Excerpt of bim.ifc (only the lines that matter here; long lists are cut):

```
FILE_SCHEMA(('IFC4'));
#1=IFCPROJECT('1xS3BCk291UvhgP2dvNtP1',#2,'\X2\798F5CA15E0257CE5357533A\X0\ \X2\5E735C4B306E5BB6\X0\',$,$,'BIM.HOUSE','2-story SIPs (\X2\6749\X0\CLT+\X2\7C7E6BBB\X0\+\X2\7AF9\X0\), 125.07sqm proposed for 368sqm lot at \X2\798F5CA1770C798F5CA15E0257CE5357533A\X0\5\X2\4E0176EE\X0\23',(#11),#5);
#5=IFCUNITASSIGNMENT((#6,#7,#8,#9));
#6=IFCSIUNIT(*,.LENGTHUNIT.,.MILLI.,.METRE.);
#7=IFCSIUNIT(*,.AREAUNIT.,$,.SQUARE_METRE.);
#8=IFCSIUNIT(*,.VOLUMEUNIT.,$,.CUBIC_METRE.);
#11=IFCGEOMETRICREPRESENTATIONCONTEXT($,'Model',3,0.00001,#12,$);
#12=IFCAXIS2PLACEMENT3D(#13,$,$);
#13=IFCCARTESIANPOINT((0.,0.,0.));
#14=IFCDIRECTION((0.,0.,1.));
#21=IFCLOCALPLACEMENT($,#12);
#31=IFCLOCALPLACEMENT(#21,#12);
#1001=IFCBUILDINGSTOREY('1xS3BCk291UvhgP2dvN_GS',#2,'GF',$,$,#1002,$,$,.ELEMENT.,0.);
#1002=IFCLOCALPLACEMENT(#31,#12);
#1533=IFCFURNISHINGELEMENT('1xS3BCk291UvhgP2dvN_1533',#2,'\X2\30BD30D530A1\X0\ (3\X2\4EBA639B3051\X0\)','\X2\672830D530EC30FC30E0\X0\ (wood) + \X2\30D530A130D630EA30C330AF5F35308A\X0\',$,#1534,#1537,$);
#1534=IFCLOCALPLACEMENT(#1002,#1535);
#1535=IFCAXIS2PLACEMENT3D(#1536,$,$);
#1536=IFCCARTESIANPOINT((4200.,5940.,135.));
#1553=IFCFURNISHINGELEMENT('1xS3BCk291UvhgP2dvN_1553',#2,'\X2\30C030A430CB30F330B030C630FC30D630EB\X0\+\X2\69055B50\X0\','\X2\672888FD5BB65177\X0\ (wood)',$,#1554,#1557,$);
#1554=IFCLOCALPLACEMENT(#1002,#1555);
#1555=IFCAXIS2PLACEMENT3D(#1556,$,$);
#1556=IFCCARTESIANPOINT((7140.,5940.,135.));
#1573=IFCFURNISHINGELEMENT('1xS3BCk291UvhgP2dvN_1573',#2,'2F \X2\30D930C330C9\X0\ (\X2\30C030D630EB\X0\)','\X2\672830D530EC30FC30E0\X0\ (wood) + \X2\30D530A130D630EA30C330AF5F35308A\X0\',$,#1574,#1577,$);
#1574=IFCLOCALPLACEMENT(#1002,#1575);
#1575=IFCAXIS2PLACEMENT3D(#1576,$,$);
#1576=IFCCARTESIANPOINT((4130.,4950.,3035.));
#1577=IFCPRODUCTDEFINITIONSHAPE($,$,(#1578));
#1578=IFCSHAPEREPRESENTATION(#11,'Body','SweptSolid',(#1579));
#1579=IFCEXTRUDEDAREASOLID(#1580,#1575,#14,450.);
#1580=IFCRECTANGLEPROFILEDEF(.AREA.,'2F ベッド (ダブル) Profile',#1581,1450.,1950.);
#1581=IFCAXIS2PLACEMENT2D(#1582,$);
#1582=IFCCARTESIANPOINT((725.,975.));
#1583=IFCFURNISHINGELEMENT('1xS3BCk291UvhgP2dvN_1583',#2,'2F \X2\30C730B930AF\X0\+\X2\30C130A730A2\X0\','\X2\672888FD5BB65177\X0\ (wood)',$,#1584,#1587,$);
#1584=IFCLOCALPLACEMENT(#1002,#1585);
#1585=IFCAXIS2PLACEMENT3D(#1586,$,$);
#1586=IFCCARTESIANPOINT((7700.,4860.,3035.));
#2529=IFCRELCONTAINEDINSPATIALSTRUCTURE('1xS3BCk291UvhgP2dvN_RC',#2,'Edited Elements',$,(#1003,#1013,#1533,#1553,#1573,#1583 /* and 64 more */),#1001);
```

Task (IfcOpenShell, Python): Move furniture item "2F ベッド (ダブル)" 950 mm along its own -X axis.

```python
import ifcopenshell
import ifcopenshell.api.geometry
import ifcopenshell.util.placement

model = ifcopenshell.open("bim.ifc")

item = model.by_guid("1xS3BCk291UvhgP2dvN_1573")
matrix = ifcopenshell.util.placement.get_local_placement(item.ObjectPlacement)
matrix[:3, 3] -= matrix[:3, 0] * 950.0
ifcopenshell.api.geometry.edit_object_placement(model, product=item, matrix=matrix, is_si=False)

print(ifcopenshell.util.placement.get_local_placement(item.ObjectPlacement).round(3) + 0.0)

model.write("bim-out.ifc")
```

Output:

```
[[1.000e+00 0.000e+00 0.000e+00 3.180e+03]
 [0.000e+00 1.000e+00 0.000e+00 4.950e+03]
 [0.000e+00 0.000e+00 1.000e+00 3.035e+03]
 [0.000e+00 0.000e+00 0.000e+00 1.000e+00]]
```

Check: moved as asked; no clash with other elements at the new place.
